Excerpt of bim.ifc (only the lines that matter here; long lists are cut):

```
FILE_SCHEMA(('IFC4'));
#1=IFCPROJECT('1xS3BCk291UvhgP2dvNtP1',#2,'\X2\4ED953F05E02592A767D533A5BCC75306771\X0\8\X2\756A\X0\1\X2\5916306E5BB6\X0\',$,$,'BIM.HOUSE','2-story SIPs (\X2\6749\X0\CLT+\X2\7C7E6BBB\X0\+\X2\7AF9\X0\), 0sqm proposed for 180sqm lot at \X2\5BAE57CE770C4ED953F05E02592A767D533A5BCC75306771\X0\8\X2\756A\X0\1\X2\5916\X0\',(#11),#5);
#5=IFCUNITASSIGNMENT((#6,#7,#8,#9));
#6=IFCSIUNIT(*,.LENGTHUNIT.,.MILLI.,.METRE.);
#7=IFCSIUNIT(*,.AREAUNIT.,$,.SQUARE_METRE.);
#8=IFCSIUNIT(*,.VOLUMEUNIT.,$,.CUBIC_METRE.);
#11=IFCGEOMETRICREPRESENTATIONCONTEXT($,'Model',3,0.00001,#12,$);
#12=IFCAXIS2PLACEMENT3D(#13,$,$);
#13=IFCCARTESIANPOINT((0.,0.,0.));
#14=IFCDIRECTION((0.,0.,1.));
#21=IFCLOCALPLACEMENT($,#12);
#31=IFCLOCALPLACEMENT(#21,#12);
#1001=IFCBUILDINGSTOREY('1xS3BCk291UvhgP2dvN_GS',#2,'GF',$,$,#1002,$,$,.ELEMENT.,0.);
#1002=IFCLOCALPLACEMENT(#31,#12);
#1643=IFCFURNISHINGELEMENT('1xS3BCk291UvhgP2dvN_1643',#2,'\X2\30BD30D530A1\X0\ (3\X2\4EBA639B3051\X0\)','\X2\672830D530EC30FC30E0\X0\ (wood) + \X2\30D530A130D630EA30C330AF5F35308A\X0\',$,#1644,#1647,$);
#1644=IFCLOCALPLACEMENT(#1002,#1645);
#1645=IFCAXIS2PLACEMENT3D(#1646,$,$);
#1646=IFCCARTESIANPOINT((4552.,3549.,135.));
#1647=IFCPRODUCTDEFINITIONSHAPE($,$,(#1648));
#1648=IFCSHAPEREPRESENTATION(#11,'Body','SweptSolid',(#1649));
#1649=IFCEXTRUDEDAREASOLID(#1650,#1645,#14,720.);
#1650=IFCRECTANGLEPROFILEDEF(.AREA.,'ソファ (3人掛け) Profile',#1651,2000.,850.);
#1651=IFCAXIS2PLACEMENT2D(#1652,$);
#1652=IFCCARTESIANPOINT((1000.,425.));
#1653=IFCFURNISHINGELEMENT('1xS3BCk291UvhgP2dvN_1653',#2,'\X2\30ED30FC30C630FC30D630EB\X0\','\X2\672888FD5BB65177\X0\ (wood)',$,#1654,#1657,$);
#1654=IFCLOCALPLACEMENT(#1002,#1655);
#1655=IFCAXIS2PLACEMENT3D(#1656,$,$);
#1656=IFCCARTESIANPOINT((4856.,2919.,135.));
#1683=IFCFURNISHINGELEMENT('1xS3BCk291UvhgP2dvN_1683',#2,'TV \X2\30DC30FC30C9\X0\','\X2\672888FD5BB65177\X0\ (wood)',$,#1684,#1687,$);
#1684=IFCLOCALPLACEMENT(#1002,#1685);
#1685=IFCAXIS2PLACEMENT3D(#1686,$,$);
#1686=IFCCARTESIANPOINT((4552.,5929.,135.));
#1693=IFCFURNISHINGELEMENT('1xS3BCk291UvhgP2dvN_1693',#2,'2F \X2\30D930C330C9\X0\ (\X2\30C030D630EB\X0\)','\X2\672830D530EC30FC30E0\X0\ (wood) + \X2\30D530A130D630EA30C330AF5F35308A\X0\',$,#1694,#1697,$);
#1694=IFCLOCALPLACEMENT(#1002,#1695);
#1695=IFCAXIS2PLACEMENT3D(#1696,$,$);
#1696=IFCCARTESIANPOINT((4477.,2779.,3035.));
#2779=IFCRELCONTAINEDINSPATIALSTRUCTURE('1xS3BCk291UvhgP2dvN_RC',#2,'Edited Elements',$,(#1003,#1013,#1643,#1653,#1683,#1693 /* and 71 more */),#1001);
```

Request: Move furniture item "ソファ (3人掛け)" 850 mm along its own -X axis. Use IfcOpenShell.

```python
import ifcopenshell
import ifcopenshell.api.geometry
import ifcopenshell.util.placement

model = ifcopenshell.open("bim.ifc")

item = model.by_id(1643)
matrix = ifcopenshell.util.placement.get_local_placement(item.ObjectPlacement)
matrix[:3, 3] -= matrix[:3, 0] * 850.0
ifcopenshell.api.geometry.edit_object_placement(model, product=item, matrix=matrix, is_si=False)

print(ifcopenshell.util.placement.get_local_placement(item.ObjectPlacement).round(3) + 0.0)

model.write("bim_updated.ifc")
```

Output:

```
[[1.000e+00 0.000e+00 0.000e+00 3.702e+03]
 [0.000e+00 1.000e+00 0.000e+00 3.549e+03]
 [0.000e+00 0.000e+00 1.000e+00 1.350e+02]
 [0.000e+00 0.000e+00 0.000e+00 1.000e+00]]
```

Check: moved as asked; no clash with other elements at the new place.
